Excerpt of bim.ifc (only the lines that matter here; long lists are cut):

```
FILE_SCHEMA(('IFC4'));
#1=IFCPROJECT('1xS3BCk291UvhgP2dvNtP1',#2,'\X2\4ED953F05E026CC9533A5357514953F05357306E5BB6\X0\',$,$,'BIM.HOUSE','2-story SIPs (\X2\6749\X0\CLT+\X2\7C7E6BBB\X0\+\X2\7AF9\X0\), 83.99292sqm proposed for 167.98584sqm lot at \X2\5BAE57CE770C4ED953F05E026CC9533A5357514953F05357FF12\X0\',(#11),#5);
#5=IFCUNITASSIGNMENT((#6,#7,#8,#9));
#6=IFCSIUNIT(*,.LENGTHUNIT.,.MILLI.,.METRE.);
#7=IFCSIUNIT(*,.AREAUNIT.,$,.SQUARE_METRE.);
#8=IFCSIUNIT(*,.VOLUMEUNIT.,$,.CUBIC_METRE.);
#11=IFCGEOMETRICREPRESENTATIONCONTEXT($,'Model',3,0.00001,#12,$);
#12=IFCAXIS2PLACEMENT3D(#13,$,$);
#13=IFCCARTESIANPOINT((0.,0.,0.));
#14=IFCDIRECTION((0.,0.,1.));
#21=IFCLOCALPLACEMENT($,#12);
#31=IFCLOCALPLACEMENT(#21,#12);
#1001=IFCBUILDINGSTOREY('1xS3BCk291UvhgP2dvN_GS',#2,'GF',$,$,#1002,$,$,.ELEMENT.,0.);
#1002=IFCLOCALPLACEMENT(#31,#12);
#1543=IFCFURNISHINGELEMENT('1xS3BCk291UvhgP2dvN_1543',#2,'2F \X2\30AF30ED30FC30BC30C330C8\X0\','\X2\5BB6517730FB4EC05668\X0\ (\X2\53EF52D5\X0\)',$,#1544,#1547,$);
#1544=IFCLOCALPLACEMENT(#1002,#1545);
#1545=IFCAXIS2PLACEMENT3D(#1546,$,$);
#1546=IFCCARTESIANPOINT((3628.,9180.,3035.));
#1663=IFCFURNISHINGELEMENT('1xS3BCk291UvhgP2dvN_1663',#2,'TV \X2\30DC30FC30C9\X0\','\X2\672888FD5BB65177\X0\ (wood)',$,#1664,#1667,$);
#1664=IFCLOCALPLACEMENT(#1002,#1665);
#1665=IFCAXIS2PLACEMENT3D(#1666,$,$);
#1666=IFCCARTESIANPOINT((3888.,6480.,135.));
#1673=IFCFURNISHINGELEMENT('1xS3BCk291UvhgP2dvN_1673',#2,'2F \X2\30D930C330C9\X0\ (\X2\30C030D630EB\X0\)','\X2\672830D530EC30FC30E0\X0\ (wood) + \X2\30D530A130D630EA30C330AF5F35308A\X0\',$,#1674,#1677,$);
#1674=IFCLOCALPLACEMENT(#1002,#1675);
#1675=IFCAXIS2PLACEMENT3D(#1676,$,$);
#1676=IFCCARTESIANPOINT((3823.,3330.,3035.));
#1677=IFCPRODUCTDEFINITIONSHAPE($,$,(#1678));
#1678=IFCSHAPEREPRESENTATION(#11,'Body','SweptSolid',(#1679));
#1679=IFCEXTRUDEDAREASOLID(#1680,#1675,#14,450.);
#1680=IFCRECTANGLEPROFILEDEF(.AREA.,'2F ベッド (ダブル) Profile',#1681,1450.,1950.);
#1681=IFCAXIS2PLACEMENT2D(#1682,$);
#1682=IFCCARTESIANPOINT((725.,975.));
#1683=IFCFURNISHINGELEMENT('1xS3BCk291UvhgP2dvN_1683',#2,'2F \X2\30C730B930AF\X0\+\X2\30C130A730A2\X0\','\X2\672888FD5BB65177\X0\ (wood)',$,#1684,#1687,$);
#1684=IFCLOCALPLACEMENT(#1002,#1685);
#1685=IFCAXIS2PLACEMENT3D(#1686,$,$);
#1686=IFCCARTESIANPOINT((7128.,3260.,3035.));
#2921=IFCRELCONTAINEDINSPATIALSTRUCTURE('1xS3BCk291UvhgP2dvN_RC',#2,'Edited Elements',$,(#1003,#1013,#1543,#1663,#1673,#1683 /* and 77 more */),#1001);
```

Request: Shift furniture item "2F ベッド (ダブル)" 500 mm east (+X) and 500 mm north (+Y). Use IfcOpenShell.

```python
import ifcopenshell
import ifcopenshell.api.geometry
import ifcopenshell.util.placement

model = ifcopenshell.open("bim.ifc")

item = model.by_guid("1xS3BCk291UvhgP2dvN_1673")
matrix = ifcopenshell.util.placement.get_local_placement(item.ObjectPlacement)
matrix[0, 3] += 500.0
matrix[1, 3] += 500.0
ifcopenshell.api.geometry.edit_object_placement(model, product=item, matrix=matrix, is_si=False)

print(ifcopenshell.util.placement.get_local_placement(item.ObjectPlacement).round(3) + 0.0)

model.write("bim_v2.ifc")
```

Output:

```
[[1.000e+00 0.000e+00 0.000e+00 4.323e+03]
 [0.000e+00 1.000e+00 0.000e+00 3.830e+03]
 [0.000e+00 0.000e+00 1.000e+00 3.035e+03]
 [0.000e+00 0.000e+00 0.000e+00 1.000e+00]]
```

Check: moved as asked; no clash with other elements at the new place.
